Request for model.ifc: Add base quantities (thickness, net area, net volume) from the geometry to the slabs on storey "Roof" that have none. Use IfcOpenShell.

First a look at what the model holds.

```python
import ifcopenshell
import ifcopenshell.util.element
import ifcopenshell.util.unit

model = ifcopenshell.open("model.ifc")
print(model.schema)
for unit_type in ("LENGTHUNIT", "AREAUNIT", "VOLUMEUNIT"):
    print(unit_type, ifcopenshell.util.unit.calculate_unit_scale(model, unit_type))
storey = next(s for s in model.by_type("IfcBuildingStorey") if s.Name == "Roof")
slabs = [e for e in ifcopenshell.util.element.get_decomposition(storey) if e.is_a("IfcSlab")]
for e in sorted(slabs, key=lambda e: e.id()):
    print(e.id(), e.is_a(), e.Name, list(ifcopenshell.util.element.get_psets(e, qtos_only=True)), sep=" | ")
```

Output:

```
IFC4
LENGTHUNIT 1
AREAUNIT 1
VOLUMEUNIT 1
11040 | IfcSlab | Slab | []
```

```python
import ifcopenshell
import ifcopenshell.api.pset
import ifcopenshell.geom
import ifcopenshell.util.element
import ifcopenshell.util.shape
import ifcopenshell.util.unit

model = ifcopenshell.open("model.ifc")
unit_scale = ifcopenshell.util.unit.calculate_unit_scale(model)
area_scale = ifcopenshell.util.unit.calculate_unit_scale(model, "AREAUNIT")
volume_scale = ifcopenshell.util.unit.calculate_unit_scale(model, "VOLUMEUNIT")
settings = ifcopenshell.geom.settings()

storey = next(s for s in model.by_type("IfcBuildingStorey") if s.Name == "Roof")
slabs = [e for e in ifcopenshell.util.element.get_decomposition(storey) if e.is_a("IfcSlab")]

for e in sorted(slabs, key=lambda e: e.id()):
    if ifcopenshell.util.element.get_psets(e, qtos_only=True, should_inherit=False):
        continue
    # Geometry comes back in metres, in the element's own axes.
    shape = ifcopenshell.geom.create_shape(settings, e)
    values = {
        "Width": ifcopenshell.util.shape.get_z(shape.geometry) / unit_scale,
        "NetArea": ifcopenshell.util.shape.get_footprint_area(shape.geometry) / area_scale,
        "NetVolume": ifcopenshell.util.shape.get_volume(shape.geometry) / volume_scale,
    }
    qto = ifcopenshell.api.pset.add_qto(model, product=e, name="Qto_SlabBaseQuantities")
    ifcopenshell.api.pset.edit_qto(model, qto=qto, properties=values)
    print(e.id(), {k: round(v, 3) for k, v in values.items()})

model.write("model-out.ifc")
```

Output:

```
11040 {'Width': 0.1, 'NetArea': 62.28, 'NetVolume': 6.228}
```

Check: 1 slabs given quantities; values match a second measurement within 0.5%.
